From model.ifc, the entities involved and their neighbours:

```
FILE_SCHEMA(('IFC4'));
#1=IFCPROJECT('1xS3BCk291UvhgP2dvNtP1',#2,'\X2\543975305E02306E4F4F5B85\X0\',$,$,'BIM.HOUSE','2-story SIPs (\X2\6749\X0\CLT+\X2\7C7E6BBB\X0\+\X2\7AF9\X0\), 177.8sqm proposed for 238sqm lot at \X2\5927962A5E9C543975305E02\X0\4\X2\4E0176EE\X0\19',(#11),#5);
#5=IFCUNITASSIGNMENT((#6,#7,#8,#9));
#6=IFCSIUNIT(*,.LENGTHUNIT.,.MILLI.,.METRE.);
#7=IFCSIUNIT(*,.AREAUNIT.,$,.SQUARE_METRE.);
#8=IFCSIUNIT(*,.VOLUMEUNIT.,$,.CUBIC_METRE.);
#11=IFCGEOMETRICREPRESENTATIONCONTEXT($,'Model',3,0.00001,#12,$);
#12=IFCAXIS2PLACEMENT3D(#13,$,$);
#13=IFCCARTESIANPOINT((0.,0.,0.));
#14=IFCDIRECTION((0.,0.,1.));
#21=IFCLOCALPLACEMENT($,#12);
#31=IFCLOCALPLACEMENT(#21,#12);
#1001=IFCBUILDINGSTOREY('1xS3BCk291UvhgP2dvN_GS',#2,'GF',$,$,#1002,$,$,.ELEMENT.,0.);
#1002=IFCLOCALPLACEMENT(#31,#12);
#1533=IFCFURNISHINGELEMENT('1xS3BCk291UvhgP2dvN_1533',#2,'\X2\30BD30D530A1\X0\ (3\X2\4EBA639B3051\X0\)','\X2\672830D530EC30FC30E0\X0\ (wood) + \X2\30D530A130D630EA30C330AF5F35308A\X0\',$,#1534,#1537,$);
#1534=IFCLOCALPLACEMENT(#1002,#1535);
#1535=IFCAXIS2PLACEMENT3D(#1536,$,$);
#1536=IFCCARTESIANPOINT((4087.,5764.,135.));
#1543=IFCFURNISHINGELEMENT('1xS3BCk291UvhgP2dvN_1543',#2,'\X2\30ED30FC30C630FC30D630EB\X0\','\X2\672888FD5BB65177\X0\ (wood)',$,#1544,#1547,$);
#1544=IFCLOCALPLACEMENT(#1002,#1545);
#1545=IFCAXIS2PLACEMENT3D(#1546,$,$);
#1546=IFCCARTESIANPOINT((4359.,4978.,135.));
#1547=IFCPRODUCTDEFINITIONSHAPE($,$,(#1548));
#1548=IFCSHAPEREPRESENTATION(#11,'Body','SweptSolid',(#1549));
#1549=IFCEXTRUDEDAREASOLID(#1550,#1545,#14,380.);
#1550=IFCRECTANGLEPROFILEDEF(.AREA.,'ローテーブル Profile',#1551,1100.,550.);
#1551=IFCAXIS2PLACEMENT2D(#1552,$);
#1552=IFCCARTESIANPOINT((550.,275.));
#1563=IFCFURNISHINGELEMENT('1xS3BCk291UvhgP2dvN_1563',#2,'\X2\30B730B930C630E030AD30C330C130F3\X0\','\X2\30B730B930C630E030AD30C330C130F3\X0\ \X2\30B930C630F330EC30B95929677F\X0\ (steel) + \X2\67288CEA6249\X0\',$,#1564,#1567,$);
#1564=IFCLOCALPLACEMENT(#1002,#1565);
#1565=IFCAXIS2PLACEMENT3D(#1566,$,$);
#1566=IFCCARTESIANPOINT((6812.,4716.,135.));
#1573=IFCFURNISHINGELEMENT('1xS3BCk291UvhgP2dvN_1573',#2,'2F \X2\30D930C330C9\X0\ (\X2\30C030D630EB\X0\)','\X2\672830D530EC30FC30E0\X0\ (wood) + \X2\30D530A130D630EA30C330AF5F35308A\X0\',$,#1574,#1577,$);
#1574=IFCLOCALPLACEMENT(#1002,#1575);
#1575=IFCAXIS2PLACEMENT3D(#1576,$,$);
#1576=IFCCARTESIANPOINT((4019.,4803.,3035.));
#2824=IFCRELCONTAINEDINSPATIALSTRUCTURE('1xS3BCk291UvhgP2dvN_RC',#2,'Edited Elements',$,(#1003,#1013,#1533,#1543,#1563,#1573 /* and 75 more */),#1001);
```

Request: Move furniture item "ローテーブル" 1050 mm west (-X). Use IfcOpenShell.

```python
import ifcopenshell
import ifcopenshell.api.geometry
import ifcopenshell.util.placement

model = ifcopenshell.open("model.ifc")

item = model.by_id(1543)
matrix = ifcopenshell.util.placement.get_local_placement(item.ObjectPlacement)
matrix[0, 3] -= 1050.0
ifcopenshell.api.geometry.edit_object_placement(model, product=item, matrix=matrix, is_si=False)

print(ifcopenshell.util.placement.get_local_placement(item.ObjectPlacement).round(3) + 0.0)

model.write("model_v2.ifc")
```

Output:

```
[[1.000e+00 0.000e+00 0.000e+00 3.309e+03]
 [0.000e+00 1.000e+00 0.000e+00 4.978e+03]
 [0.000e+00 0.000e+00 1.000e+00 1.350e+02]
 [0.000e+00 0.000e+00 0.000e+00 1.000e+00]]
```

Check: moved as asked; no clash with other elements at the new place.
